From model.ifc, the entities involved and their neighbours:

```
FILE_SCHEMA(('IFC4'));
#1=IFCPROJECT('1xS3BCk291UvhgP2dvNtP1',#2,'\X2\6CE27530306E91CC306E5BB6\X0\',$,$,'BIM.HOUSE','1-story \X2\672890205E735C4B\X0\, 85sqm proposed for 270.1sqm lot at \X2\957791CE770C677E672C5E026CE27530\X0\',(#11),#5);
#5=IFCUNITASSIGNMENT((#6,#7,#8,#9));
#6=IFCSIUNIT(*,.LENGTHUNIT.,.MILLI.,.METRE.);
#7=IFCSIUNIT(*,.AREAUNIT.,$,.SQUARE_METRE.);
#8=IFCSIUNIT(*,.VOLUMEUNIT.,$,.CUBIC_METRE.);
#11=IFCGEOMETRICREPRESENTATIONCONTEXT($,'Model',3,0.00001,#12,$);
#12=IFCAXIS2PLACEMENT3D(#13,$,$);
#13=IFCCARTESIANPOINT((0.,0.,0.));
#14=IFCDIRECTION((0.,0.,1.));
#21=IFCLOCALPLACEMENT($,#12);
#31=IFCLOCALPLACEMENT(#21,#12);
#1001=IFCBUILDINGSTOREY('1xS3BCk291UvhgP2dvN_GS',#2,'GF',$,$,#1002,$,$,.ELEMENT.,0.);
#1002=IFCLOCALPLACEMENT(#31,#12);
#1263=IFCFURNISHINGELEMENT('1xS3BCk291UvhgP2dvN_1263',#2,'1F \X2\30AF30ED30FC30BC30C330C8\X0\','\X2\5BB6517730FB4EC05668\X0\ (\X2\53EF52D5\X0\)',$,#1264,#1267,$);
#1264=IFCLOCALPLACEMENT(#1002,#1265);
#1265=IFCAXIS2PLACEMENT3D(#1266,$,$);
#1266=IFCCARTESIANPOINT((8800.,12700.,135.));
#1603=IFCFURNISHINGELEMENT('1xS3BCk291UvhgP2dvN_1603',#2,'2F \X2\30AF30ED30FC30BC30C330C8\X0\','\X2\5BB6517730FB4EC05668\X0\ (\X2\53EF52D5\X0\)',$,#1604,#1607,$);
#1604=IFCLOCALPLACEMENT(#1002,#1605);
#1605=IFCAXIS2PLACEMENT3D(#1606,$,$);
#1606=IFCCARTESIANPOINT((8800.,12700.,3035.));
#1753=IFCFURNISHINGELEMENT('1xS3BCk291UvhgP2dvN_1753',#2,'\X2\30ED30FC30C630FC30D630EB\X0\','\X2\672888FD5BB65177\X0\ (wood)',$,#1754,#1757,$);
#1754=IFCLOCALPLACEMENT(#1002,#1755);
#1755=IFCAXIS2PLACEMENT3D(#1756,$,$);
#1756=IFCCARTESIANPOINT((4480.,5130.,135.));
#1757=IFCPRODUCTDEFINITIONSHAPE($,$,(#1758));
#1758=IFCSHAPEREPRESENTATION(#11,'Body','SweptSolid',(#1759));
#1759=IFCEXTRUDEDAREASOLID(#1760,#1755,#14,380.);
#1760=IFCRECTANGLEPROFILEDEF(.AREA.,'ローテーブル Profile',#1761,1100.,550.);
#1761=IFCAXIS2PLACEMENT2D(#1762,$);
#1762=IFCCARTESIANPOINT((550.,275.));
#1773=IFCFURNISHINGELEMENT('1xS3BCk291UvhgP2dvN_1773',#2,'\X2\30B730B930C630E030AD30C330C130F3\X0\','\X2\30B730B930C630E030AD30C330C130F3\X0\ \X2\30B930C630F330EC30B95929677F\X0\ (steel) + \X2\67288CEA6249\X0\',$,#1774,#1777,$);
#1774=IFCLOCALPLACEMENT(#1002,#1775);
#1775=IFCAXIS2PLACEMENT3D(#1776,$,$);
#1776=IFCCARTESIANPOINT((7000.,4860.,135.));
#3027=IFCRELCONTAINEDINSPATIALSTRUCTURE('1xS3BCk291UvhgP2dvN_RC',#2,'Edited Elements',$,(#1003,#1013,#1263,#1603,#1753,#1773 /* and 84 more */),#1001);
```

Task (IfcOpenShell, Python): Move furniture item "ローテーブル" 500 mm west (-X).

```python
import ifcopenshell
import ifcopenshell.api.geometry
import ifcopenshell.util.placement
import ifcopenshell.util.unit

model = ifcopenshell.open("model.ifc")
unit_scale = ifcopenshell.util.unit.calculate_unit_scale(model)

item = model.by_id(1753)
matrix = ifcopenshell.util.placement.get_local_placement(item.ObjectPlacement)
matrix[0, 3] -= 0.5 / unit_scale
ifcopenshell.api.geometry.edit_object_placement(model, product=item, matrix=matrix, is_si=False)

print(ifcopenshell.util.placement.get_local_placement(item.ObjectPlacement).round(3) + 0.0)

model.write("model_rev.ifc")
```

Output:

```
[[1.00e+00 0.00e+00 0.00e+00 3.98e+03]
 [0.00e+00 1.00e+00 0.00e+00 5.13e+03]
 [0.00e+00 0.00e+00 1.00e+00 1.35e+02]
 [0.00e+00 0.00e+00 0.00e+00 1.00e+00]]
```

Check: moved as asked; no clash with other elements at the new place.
